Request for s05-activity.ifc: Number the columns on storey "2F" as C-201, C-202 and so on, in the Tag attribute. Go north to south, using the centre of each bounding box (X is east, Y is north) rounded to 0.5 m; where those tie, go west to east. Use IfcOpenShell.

First a look at what the model holds.

```python
import ifcopenshell
import ifcopenshell.util.element
import ifcopenshell.util.placement

model = ifcopenshell.open("s05-activity.ifc")
print(model.schema)
storey = next(s for s in model.by_type("IfcBuildingStorey") if s.Name == "2F")
columns = [e for e in ifcopenshell.util.element.get_decomposition(storey) if e.is_a("IfcColumn")]
for e in sorted(columns, key=lambda e: e.id()):
    origin = ifcopenshell.util.placement.get_local_placement(e.ObjectPlacement)[:3, 3]
    print(e.id(), e.Tag, e.Name, origin.round(2) + 0.0, sep=" | ")
```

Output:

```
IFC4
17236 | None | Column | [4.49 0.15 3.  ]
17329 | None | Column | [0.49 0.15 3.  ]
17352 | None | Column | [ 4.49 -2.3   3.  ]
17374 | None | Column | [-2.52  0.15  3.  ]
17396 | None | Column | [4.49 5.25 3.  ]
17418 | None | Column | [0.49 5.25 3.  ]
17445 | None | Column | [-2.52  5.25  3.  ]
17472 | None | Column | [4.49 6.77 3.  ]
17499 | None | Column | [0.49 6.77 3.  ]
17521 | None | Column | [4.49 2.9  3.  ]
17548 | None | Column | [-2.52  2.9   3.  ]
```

```python
import ifcopenshell
import ifcopenshell.geom
import ifcopenshell.util.element
import ifcopenshell.util.shape

model = ifcopenshell.open("s05-activity.ifc")
settings = ifcopenshell.geom.settings()
settings.set("use-world-coords", True)


def centre(element):
    shape = ifcopenshell.geom.create_shape(settings, element)
    return ifcopenshell.util.shape.get_bbox_centroid(shape.geometry)


storey = next(s for s in model.by_type("IfcBuildingStorey") if s.Name == "2F")
columns = [e for e in ifcopenshell.util.element.get_decomposition(storey) if e.is_a("IfcColumn")]

# Insertion points can sit at a corner or the storey origin, so sort by the geometry (in metres).
centres = {e: centre(e) for e in columns}
columns.sort(key=lambda e: (-round(centres[e][1] / 0.5), centres[e][0]))

for i, e in enumerate(columns, start=1):
    number = f"C-2{i:02d}"
    e.Tag = number
    print(e.id(), number)

model.write("s05-activity_v2.ifc")
```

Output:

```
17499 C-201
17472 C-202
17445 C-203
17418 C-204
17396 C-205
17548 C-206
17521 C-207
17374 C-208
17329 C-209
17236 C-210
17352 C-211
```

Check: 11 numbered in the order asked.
